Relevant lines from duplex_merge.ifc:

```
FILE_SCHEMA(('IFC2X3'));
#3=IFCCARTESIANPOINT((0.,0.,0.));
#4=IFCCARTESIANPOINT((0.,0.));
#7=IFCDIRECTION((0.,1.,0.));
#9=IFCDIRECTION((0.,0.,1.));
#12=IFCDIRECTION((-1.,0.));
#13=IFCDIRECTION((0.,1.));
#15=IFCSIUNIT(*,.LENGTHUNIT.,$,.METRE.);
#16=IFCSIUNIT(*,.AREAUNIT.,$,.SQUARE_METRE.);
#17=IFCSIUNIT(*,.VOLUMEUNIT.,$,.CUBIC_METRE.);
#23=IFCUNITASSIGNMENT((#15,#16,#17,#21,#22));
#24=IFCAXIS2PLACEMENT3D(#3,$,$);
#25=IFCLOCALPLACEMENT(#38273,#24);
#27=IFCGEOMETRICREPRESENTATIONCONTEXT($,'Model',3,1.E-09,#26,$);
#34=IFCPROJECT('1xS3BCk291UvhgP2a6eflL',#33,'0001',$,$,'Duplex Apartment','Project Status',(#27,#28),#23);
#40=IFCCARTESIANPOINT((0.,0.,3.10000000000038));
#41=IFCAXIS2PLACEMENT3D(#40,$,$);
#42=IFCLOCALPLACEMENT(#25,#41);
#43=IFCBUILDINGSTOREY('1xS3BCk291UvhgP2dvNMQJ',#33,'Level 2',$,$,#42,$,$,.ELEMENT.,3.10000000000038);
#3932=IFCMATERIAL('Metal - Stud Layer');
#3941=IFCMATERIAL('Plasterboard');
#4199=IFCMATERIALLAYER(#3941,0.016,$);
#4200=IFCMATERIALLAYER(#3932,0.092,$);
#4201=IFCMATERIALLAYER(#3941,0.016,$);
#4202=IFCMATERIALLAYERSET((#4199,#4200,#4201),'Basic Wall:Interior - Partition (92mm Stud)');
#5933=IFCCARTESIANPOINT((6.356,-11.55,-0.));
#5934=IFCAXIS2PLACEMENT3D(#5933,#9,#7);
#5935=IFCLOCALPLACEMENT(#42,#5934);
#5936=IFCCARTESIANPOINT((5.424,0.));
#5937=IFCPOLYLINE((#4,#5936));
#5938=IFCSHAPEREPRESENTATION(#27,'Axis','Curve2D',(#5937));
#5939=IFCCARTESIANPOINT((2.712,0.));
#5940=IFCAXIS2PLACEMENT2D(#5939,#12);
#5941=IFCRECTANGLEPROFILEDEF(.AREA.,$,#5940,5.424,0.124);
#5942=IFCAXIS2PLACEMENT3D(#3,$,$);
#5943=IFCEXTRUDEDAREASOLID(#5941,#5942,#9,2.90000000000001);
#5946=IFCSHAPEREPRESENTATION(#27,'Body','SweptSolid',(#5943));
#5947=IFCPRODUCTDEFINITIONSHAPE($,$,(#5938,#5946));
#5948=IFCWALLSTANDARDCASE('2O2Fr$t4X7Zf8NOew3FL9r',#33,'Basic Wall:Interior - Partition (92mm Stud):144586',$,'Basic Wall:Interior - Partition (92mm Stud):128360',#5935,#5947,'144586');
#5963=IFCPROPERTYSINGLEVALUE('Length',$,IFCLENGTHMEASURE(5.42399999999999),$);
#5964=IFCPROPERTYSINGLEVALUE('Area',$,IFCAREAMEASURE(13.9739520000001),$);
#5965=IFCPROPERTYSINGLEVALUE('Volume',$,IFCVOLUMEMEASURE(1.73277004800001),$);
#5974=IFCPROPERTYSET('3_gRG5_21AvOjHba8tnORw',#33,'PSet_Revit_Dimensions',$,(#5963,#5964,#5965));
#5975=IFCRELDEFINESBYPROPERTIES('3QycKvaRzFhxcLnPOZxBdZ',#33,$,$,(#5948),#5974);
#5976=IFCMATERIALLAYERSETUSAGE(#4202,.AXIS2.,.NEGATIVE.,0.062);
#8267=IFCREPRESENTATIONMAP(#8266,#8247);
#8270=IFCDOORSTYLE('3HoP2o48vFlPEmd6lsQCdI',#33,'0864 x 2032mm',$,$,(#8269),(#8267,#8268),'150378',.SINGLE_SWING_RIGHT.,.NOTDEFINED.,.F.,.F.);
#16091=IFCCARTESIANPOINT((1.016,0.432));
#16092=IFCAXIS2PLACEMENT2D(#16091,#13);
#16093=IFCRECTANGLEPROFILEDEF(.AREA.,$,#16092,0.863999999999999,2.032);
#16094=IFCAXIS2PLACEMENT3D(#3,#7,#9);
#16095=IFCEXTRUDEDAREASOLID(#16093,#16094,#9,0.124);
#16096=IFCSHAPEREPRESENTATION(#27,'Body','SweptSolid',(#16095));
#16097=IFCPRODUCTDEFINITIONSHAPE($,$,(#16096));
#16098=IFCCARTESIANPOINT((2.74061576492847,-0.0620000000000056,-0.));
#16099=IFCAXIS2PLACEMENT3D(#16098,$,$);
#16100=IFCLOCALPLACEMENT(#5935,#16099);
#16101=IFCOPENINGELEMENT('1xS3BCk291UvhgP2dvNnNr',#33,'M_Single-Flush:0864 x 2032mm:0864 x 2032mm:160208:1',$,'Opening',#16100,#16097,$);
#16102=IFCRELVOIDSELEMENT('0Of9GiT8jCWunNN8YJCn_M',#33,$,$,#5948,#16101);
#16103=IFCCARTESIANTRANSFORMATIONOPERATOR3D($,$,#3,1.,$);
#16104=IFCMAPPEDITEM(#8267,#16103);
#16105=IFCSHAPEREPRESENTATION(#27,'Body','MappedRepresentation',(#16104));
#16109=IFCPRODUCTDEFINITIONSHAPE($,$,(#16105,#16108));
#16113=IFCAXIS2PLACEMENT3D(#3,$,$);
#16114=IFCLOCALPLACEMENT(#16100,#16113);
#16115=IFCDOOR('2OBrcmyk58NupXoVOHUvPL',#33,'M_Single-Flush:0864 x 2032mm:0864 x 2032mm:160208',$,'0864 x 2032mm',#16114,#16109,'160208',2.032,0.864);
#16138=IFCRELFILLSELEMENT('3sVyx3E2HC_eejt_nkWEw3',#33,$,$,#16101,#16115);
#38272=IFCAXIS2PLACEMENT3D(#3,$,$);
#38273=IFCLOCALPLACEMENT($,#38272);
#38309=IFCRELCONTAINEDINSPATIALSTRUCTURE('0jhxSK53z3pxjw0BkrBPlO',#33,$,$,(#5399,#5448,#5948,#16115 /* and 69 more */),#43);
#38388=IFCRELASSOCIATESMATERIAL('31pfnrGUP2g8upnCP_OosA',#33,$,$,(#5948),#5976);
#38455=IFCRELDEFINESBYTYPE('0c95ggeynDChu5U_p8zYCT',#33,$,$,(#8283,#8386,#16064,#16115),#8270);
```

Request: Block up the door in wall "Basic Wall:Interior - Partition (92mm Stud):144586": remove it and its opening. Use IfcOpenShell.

```python
import ifcopenshell
import ifcopenshell.api.feature
import ifcopenshell.api.pset
import ifcopenshell.api.root
import ifcopenshell.geom
import ifcopenshell.util.element
import ifcopenshell.util.shape
import ifcopenshell.util.unit

model = ifcopenshell.open("duplex_merge.ifc")
area_scale = ifcopenshell.util.unit.calculate_unit_scale(model, "AREAUNIT")
volume_scale = ifcopenshell.util.unit.calculate_unit_scale(model, "VOLUMEUNIT")
settings = ifcopenshell.geom.settings()


def volume(element):
    """Net volume in cubic metres, openings subtracted."""
    shape = ifcopenshell.geom.create_shape(settings, element)
    return ifcopenshell.util.shape.get_volume(shape.geometry)


door = model.by_guid("2OBrcmyk58NupXoVOHUvPL")
opening = door.FillsVoids[0].RelatingOpeningElement
wall = opening.VoidsElements[0].RelatingBuildingElement
before = volume(wall)

ifcopenshell.api.root.remove_product(model, product=door)
ifcopenshell.api.feature.remove_feature(model, feature=opening)

after = volume(wall)
thickness = 0.124  # wall thickness in metres

# Update the wall's stored quantities.
pset = model.by_id(ifcopenshell.util.element.get_pset(wall, "PSet_Revit_Dimensions", should_inherit=False)["id"])
ifcopenshell.api.pset.edit_pset(model, pset=pset, properties={
    "Area": model.create_entity("IfcAreaMeasure", after / thickness / area_scale),
    "Volume": model.create_entity("IfcVolumeMeasure", after / volume_scale),
})

print(f"wall volume {before:.3f} -> {after:.3f} m3")

model.write("duplex_merge_edited.ifc")
```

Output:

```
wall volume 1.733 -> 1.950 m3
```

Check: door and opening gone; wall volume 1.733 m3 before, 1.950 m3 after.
